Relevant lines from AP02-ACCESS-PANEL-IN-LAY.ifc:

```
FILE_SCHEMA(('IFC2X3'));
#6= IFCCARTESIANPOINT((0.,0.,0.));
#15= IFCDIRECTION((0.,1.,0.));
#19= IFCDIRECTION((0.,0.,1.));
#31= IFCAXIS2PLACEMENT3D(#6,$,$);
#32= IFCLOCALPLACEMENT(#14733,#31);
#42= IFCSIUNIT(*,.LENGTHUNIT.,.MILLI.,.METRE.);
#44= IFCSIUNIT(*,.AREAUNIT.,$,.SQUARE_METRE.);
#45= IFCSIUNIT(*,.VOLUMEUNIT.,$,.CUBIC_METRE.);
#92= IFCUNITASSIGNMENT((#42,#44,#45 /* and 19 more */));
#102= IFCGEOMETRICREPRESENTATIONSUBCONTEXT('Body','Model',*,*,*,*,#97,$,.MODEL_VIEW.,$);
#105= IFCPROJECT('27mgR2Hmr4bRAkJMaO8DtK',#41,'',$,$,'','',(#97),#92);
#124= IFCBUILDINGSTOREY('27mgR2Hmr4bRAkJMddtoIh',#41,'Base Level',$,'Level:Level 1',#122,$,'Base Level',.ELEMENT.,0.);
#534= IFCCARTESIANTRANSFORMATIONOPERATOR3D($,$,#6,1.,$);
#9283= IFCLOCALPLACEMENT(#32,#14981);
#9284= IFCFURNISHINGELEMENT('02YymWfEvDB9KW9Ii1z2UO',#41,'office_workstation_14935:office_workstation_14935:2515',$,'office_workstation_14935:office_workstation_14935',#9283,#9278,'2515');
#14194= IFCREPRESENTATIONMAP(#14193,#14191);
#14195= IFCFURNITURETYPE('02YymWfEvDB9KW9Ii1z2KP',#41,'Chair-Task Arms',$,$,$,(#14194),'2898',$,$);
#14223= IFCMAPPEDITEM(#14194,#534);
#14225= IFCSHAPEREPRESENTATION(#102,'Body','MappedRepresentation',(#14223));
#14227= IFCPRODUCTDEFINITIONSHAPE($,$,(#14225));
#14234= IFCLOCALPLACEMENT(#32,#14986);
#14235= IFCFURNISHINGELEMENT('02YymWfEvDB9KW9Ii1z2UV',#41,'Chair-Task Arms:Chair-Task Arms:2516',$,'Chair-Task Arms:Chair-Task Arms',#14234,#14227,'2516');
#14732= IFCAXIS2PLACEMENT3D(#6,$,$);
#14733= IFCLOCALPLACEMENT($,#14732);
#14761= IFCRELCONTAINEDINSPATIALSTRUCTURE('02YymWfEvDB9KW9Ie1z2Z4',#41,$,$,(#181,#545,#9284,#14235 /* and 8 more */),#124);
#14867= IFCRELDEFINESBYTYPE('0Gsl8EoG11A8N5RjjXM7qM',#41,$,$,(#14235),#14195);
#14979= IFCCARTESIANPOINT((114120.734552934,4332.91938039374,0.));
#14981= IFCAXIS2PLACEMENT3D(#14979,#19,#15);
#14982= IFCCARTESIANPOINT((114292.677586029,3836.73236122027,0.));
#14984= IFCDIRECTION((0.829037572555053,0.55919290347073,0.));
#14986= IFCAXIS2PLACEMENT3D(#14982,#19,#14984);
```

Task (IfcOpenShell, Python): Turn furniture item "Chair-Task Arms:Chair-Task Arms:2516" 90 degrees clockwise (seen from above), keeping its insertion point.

```python
import ifcopenshell
import ifcopenshell.api.geometry
import ifcopenshell.util.placement

model = ifcopenshell.open("AP02-ACCESS-PANEL-IN-LAY.ifc")

item = model.by_id(14235)
matrix = ifcopenshell.util.placement.get_local_placement(item.ObjectPlacement)
matrix = matrix @ ifcopenshell.util.placement.rotation(-90, "Z")
ifcopenshell.api.geometry.edit_object_placement(model, product=item, matrix=matrix, is_si=False)

print(ifcopenshell.util.placement.get_local_placement(item.ObjectPlacement).round(3) + 0.0)

model.write("AP02-ACCESS-PANEL-IN-LAY_rev.ifc")
```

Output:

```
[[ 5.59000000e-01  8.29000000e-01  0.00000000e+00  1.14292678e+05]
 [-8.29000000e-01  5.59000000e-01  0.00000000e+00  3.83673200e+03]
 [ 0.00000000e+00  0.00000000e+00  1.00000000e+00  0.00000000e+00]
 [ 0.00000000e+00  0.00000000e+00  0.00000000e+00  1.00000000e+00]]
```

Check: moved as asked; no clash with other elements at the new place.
